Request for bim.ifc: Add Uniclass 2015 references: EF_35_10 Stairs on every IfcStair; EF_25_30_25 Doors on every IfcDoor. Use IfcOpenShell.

First a look at what the model holds.

```python
import ifcopenshell

model = ifcopenshell.open("bim.ifc")
print(model.schema)
print("classifications:", [c.Name for c in model.by_type("IfcClassification")])
for ifc_class in ("IfcDoor", "IfcRoof", "IfcStair", "IfcWall", "IfcWindow"):
    print(ifc_class, len(model.by_type(ifc_class)))
```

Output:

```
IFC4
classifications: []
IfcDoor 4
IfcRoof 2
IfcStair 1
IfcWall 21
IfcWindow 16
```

```python
import ifcopenshell
import ifcopenshell.api.classification

model = ifcopenshell.open("bim.ifc")

system = ifcopenshell.api.classification.add_classification(model, classification="Uniclass 2015")

codes = {
    "IfcStair": ("EF_35_10", "Stairs"),
    "IfcDoor": ("EF_25_30_25", "Doors"),
}
for ifc_class, (code, name) in codes.items():
    products = model.by_type(ifc_class)
    ifcopenshell.api.classification.add_reference(
        model, products=products, classification=system, identification=code, name=name
    )
    print(code, len(products))

model.write("bim_edited.ifc")
```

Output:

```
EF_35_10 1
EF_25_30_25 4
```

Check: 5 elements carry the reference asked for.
